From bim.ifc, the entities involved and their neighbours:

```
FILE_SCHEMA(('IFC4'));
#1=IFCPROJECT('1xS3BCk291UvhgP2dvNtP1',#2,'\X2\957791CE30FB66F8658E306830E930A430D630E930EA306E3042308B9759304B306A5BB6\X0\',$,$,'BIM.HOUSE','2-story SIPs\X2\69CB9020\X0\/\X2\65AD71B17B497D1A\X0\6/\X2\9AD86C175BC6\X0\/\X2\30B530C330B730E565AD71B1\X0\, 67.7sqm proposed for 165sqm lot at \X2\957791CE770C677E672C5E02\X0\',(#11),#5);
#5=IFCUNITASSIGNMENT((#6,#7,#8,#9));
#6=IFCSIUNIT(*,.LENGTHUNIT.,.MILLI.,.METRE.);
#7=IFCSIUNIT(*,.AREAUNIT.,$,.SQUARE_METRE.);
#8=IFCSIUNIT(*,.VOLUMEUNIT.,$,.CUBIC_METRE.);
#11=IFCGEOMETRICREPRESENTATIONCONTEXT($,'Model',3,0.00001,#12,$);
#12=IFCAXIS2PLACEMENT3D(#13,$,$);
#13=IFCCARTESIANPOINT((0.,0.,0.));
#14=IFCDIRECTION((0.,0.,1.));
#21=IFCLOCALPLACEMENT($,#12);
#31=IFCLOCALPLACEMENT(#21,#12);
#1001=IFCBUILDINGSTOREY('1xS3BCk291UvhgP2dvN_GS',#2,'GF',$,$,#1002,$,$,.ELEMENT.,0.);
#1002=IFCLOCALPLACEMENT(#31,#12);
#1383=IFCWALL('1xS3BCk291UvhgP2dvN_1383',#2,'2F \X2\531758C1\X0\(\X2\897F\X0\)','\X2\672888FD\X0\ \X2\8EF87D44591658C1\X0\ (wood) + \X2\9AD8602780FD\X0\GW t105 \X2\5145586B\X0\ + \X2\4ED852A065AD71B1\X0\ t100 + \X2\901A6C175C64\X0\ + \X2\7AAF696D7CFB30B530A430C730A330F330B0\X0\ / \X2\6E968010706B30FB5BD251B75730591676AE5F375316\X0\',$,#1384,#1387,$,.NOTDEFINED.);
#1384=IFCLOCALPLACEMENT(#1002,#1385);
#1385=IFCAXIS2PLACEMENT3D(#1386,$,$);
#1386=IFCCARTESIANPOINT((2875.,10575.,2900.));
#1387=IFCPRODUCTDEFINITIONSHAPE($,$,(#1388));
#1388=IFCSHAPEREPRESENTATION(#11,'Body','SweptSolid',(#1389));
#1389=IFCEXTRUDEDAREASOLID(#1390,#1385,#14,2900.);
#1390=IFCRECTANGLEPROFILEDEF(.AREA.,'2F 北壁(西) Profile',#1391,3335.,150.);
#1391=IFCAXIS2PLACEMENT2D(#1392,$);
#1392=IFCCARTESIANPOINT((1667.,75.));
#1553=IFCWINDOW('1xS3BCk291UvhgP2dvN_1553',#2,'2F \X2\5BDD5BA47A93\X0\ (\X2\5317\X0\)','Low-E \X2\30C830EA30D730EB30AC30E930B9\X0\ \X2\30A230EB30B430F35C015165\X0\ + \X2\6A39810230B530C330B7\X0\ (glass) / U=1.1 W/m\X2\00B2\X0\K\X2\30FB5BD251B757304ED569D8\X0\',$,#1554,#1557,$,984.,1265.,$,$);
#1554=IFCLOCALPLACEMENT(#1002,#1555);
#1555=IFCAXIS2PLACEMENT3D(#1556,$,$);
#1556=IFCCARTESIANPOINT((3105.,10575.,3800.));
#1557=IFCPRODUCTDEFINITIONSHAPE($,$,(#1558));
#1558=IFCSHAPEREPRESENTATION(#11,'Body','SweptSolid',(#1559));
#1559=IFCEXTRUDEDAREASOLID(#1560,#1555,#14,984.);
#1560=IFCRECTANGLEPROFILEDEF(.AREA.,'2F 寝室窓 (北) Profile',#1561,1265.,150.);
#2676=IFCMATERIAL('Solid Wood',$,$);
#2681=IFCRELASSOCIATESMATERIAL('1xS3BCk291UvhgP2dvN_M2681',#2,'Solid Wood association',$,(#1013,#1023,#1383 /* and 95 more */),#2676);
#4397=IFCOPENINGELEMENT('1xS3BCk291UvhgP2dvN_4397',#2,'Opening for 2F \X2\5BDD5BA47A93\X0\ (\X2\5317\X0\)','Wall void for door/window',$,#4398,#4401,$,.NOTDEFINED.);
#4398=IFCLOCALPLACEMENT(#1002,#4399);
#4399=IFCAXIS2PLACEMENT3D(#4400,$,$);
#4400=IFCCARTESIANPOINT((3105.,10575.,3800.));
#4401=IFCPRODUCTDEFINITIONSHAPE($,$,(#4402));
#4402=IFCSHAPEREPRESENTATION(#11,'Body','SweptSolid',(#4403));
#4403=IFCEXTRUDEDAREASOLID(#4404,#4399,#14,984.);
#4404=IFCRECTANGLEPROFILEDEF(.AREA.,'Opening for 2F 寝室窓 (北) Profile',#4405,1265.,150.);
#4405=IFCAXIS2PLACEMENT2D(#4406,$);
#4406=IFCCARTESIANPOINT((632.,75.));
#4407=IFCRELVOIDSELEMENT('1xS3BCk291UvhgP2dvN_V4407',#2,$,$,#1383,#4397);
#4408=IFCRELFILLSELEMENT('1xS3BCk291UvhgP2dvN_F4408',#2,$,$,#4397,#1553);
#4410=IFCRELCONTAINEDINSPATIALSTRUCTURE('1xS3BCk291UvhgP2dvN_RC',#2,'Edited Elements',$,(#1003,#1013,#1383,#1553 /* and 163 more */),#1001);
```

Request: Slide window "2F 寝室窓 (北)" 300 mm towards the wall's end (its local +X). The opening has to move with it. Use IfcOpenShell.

```python
import ifcopenshell
import ifcopenshell.api.geometry
import ifcopenshell.util.placement
import ifcopenshell.util.unit

model = ifcopenshell.open("bim.ifc")
unit_scale = ifcopenshell.util.unit.calculate_unit_scale(model)

window = model.by_id(1553)
opening = window.FillsVoids[0].RelatingOpeningElement
wall = opening.VoidsElements[0].RelatingBuildingElement

wall_matrix = ifcopenshell.util.placement.get_local_placement(wall.ObjectPlacement)
shift = wall_matrix[:3, 0] * 0.3 / unit_scale
before = ifcopenshell.util.placement.get_local_placement(window.ObjectPlacement)[:3, 3].copy()

# The window is not placed relative to its opening, so move both.
for product in (opening, window):
    matrix = ifcopenshell.util.placement.get_local_placement(product.ObjectPlacement)
    matrix[:3, 3] += shift
    ifcopenshell.api.geometry.edit_object_placement(model, product=product, matrix=matrix, is_si=False)

after = ifcopenshell.util.placement.get_local_placement(window.ObjectPlacement)[:3, 3]
print("window moved by", (after - before).round(3) + 0.0)

model.write("bim_updated.ifc")
```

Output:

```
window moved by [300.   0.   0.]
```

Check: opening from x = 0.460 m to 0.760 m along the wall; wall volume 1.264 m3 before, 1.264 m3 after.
